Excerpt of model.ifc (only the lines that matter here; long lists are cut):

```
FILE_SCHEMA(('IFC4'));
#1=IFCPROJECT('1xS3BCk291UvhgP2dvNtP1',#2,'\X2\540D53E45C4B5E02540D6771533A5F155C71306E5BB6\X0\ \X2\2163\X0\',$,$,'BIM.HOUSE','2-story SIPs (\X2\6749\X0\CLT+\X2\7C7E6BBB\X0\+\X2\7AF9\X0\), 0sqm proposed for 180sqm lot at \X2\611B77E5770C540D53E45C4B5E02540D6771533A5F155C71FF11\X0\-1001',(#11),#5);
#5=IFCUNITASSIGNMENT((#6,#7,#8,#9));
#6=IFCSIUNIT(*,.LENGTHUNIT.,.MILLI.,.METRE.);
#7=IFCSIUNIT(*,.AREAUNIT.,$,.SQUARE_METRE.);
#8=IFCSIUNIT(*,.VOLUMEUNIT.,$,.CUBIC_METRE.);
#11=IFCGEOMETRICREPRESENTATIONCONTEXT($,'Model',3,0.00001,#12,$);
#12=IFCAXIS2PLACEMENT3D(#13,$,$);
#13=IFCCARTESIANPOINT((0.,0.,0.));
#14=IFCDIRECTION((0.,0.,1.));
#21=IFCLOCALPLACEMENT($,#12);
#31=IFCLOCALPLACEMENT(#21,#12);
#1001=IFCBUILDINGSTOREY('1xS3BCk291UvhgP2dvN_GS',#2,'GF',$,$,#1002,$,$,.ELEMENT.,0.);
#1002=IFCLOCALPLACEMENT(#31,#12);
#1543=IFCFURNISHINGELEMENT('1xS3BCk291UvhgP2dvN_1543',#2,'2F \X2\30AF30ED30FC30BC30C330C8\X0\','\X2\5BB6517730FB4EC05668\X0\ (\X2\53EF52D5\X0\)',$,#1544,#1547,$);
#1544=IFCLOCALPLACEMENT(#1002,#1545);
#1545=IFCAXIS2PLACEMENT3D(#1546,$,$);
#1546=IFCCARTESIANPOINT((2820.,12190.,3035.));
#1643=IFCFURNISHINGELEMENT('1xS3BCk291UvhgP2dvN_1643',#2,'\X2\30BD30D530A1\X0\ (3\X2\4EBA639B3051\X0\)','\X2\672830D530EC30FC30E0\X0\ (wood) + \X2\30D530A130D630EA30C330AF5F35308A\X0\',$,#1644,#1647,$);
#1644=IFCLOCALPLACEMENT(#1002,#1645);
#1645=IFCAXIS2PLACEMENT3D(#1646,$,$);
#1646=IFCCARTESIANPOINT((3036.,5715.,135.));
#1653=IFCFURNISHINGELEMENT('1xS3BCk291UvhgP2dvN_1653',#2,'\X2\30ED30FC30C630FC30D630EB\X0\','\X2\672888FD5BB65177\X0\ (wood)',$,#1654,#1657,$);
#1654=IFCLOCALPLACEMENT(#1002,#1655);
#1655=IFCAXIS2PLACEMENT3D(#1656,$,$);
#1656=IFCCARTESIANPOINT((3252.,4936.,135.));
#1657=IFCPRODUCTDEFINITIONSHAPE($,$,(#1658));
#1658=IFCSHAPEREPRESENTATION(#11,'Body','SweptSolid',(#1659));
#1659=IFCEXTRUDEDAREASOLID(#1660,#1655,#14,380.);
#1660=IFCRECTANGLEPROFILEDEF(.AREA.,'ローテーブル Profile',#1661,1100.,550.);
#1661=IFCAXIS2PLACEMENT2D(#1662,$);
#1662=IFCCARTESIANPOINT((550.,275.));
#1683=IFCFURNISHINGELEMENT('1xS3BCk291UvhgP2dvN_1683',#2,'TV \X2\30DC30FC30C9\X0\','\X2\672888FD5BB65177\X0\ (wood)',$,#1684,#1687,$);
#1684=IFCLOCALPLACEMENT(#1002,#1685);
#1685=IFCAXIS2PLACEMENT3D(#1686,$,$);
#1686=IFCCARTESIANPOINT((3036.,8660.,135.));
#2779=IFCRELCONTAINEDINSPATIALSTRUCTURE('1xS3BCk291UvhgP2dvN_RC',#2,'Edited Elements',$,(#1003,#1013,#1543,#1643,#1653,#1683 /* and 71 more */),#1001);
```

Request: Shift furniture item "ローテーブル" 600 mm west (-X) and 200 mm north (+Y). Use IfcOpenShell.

```python
import ifcopenshell
import ifcopenshell.api.geometry
import ifcopenshell.util.placement
import ifcopenshell.util.unit

model = ifcopenshell.open("model.ifc")
unit_scale = ifcopenshell.util.unit.calculate_unit_scale(model)

item = model.by_guid("1xS3BCk291UvhgP2dvN_1653")
matrix = ifcopenshell.util.placement.get_local_placement(item.ObjectPlacement)
matrix[0, 3] -= 0.6 / unit_scale
matrix[1, 3] += 0.2 / unit_scale
ifcopenshell.api.geometry.edit_object_placement(model, product=item, matrix=matrix, is_si=False)

print(ifcopenshell.util.placement.get_local_placement(item.ObjectPlacement).round(3) + 0.0)

model.write("model_updated.ifc")
```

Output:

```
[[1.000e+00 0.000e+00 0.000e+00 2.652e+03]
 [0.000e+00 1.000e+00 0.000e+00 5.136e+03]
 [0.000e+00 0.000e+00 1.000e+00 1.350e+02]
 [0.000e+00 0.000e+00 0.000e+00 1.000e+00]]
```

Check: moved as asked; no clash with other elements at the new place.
